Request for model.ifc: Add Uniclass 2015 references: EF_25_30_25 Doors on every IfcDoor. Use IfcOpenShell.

First a look at what the model holds.

```python
import ifcopenshell

model = ifcopenshell.open("model.ifc")
print(model.schema)
print("classifications:", [c.Name for c in model.by_type("IfcClassification")])
for ifc_class in ("IfcDoor", "IfcRoof", "IfcStair", "IfcWall", "IfcWindow"):
    print(ifc_class, len(model.by_type(ifc_class)))
```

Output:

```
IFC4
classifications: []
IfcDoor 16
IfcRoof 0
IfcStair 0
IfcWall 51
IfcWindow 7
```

```python
import ifcopenshell
import ifcopenshell.api.classification

model = ifcopenshell.open("model.ifc")

system = ifcopenshell.api.classification.add_classification(model, classification="Uniclass 2015")

codes = {
    "IfcDoor": ("EF_25_30_25", "Doors"),
}
for ifc_class, (code, name) in codes.items():
    products = model.by_type(ifc_class)
    ifcopenshell.api.classification.add_reference(
        model, products=products, classification=system, identification=code, name=name
    )
    print(code, len(products))

model.write("model_rev.ifc")
```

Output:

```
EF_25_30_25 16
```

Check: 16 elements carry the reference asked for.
